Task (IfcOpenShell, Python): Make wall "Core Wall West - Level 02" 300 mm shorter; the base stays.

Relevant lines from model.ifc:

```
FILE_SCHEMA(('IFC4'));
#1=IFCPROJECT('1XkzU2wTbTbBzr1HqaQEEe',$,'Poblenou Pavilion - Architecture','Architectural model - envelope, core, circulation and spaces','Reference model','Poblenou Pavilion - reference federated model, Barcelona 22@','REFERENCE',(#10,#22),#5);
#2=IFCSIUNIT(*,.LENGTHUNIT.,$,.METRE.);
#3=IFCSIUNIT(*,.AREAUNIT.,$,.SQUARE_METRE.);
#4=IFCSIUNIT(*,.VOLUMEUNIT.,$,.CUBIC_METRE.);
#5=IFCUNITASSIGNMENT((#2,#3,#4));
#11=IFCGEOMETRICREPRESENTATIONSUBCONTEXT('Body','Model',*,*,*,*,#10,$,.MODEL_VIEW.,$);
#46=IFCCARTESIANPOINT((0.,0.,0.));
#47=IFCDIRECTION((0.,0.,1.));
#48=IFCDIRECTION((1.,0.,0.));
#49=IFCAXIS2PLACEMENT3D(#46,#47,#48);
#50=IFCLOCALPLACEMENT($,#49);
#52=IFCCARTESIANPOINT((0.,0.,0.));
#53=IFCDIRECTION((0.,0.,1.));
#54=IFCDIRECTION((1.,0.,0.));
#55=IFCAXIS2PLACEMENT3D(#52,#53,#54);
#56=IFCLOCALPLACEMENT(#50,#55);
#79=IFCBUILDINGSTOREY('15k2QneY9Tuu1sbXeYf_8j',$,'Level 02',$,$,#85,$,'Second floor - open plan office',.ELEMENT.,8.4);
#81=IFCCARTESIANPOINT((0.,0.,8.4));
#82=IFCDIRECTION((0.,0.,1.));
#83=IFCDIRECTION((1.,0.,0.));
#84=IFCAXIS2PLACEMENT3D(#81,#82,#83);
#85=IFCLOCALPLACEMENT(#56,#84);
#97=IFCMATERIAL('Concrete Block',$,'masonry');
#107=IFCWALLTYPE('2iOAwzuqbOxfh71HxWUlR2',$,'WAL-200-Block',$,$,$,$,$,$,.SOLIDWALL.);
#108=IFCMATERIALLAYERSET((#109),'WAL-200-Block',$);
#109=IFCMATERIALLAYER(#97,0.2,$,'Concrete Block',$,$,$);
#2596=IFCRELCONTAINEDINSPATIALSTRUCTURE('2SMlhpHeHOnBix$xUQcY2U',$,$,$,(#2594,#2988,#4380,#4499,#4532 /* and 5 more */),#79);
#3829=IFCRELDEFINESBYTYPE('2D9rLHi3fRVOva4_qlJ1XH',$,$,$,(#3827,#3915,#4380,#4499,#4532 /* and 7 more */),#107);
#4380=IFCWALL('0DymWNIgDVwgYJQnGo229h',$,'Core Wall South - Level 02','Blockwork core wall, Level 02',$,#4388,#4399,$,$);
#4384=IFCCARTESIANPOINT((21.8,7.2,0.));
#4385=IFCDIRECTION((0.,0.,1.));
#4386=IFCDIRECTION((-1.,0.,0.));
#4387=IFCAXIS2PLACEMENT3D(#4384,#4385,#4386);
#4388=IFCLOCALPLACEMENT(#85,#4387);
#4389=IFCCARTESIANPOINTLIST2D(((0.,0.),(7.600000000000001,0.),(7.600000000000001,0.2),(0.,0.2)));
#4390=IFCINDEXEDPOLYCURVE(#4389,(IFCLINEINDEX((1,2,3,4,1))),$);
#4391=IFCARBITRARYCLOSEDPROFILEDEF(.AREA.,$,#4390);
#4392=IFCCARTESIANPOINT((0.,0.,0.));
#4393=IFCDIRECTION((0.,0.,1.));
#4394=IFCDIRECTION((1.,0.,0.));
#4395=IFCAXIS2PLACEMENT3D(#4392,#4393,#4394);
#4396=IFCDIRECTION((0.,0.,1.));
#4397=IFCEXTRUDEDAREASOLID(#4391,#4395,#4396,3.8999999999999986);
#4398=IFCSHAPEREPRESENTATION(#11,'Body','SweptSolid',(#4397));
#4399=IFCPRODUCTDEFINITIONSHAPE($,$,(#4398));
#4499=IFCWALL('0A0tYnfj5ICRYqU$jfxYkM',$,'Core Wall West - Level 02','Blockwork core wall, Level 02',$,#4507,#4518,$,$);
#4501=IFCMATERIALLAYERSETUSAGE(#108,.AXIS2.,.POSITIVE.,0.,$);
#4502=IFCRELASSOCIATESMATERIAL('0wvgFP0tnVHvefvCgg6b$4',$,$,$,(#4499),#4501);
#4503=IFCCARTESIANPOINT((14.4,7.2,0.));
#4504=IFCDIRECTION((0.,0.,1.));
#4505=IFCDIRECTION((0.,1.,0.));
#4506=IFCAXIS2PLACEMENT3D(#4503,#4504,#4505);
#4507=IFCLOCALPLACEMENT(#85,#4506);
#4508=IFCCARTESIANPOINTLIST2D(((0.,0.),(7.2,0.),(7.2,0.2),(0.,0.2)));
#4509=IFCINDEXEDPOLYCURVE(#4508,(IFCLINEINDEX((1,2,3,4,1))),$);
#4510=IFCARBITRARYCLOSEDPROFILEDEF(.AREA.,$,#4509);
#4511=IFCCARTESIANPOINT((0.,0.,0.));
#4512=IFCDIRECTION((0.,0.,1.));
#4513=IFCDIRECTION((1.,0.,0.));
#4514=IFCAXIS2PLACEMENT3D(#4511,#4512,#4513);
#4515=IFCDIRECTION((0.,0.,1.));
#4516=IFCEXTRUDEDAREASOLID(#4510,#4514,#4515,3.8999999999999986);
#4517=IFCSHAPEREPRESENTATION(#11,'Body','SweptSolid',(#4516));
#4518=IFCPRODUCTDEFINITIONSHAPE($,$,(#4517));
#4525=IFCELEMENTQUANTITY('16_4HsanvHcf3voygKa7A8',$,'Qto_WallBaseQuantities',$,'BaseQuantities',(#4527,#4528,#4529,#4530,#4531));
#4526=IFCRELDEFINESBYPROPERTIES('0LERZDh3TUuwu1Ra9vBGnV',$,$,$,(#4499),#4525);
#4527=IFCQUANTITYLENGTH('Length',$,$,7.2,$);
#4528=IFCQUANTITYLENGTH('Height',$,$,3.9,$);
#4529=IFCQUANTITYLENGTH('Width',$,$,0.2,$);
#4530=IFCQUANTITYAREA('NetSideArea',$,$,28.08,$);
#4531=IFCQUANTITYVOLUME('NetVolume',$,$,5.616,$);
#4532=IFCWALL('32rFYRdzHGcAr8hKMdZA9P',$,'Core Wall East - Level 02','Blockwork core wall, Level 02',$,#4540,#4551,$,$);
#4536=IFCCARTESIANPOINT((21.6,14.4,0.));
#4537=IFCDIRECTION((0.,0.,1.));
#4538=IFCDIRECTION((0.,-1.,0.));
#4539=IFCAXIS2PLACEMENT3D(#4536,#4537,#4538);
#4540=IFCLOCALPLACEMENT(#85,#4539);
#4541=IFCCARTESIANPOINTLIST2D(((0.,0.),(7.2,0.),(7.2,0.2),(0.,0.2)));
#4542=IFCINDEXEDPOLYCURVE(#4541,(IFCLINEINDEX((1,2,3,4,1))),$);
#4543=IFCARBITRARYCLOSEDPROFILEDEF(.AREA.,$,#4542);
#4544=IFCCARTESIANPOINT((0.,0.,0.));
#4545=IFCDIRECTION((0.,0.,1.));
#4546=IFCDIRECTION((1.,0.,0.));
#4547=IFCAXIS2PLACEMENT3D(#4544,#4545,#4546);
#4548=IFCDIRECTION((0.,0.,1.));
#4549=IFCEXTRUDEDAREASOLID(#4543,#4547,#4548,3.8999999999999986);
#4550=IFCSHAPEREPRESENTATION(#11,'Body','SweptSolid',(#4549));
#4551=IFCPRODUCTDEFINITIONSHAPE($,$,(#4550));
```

```python
import ifcopenshell
import ifcopenshell.api.pset
import ifcopenshell.geom
import ifcopenshell.util.element
import ifcopenshell.util.representation
import ifcopenshell.util.shape
import ifcopenshell.util.unit

model = ifcopenshell.open("model.ifc")
unit_scale = ifcopenshell.util.unit.calculate_unit_scale(model)
area_scale = ifcopenshell.util.unit.calculate_unit_scale(model, "AREAUNIT")
volume_scale = ifcopenshell.util.unit.calculate_unit_scale(model, "VOLUMEUNIT")
settings = ifcopenshell.geom.settings()


def volume(element):
    """Net volume in cubic metres, openings subtracted."""
    shape = ifcopenshell.geom.create_shape(settings, element)
    return ifcopenshell.util.shape.get_volume(shape.geometry)


wall = model.by_guid("0A0tYnfj5ICRYqU$jfxYkM")
before = volume(wall)

body = ifcopenshell.util.representation.get_representation(wall, "Model", "Body")
solid = body.Items[0]
old_height = solid.Depth
solid.Depth -= 0.3 / unit_scale
after = volume(wall)
thickness = 0.2  # wall thickness in metres

# Update the stored height, areas and volumes.
qto = model.by_id(ifcopenshell.util.element.get_pset(wall, "Qto_WallBaseQuantities", should_inherit=False)["id"])
ifcopenshell.api.pset.edit_qto(model, qto=qto, properties={
    "Height": solid.Depth,
    "NetSideArea": after / thickness / area_scale,
    "NetVolume": after / volume_scale,
})

print(f"height {old_height:g} -> {solid.Depth:g}, volume {before:.3f} -> {after:.3f} m3")

model.write("model_v2.ifc")
```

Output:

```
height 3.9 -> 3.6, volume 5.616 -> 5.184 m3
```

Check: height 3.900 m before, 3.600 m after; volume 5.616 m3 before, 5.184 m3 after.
